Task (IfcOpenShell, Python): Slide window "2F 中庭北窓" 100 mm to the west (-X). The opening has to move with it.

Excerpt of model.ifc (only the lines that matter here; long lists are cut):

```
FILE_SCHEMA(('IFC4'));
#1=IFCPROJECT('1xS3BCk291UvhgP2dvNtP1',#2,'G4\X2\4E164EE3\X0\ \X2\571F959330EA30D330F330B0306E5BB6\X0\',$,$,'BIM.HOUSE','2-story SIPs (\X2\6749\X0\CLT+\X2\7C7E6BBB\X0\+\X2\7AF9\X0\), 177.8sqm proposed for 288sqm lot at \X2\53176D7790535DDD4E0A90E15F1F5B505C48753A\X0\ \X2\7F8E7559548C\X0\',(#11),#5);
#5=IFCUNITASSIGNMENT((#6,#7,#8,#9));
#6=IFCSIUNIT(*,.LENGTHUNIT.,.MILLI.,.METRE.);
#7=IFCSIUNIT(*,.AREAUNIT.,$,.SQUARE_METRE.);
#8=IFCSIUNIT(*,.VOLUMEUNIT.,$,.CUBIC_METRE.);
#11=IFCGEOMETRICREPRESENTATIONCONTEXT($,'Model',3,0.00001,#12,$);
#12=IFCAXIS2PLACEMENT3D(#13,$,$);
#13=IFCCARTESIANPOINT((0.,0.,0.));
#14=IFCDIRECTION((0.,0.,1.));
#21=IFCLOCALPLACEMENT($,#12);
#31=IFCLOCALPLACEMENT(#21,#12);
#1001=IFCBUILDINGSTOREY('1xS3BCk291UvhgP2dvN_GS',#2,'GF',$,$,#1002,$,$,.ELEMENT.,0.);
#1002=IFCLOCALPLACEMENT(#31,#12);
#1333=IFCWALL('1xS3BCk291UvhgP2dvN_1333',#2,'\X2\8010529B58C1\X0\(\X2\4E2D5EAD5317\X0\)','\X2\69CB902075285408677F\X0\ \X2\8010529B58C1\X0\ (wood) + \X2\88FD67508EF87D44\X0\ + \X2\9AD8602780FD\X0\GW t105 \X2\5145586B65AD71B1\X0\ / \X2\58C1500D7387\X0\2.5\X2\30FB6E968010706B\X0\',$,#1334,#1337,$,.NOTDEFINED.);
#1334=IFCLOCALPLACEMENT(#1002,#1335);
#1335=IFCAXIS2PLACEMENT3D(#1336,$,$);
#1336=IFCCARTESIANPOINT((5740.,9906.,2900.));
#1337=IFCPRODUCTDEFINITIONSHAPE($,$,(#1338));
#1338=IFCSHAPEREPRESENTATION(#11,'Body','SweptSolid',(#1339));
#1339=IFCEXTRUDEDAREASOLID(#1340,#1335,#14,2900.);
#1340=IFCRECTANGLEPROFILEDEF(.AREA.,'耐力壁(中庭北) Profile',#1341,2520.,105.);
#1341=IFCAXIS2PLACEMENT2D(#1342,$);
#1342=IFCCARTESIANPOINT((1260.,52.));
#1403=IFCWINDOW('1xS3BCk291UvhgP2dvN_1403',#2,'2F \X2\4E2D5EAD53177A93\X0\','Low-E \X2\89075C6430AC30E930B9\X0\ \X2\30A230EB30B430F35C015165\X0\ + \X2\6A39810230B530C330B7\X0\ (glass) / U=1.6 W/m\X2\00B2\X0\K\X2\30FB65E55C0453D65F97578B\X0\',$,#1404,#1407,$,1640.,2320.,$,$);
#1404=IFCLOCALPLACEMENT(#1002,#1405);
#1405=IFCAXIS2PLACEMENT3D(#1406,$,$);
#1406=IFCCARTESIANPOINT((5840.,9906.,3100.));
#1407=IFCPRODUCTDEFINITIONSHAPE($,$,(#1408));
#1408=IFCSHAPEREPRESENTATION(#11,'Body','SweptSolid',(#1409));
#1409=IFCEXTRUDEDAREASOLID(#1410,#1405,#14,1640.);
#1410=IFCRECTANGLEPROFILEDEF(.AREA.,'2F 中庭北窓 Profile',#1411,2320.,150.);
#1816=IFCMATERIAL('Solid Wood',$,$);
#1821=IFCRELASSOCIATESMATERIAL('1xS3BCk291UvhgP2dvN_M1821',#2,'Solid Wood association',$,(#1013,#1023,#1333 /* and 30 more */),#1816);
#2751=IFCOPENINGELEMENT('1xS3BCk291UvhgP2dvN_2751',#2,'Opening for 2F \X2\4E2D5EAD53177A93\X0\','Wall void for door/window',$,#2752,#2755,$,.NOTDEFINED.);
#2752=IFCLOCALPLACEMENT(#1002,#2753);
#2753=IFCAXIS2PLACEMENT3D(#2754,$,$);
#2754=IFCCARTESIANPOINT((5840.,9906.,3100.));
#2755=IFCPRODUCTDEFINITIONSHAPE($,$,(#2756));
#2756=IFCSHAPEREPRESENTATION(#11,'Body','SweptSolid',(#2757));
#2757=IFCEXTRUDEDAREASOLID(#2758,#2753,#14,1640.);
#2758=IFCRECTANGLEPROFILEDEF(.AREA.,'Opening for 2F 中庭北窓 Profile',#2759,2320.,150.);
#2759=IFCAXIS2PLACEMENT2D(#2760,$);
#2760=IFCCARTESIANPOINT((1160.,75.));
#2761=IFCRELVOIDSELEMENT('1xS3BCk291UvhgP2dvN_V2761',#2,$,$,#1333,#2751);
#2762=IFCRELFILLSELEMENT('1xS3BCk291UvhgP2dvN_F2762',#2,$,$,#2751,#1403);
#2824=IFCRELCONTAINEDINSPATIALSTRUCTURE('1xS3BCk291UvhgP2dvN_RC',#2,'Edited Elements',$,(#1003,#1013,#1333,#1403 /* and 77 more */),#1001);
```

```python
import ifcopenshell
import ifcopenshell.api.geometry
import ifcopenshell.util.placement

model = ifcopenshell.open("model.ifc")

window = model.by_id(1403)
opening = window.FillsVoids[0].RelatingOpeningElement
wall = opening.VoidsElements[0].RelatingBuildingElement

wall_matrix = ifcopenshell.util.placement.get_local_placement(wall.ObjectPlacement)
shift = wall_matrix[:3, 0] * -100.0
before = ifcopenshell.util.placement.get_local_placement(window.ObjectPlacement)[:3, 3].copy()

# The window is not placed relative to its opening, so move both.
for product in (opening, window):
    matrix = ifcopenshell.util.placement.get_local_placement(product.ObjectPlacement)
    matrix[:3, 3] += shift
    ifcopenshell.api.geometry.edit_object_placement(model, product=product, matrix=matrix, is_si=False)

after = ifcopenshell.util.placement.get_local_placement(window.ObjectPlacement)[:3, 3]
print("window moved by", (after - before).round(3) + 0.0)

model.write("model_v2.ifc")
```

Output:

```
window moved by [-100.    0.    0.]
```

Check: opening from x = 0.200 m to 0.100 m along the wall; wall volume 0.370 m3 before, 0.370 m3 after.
